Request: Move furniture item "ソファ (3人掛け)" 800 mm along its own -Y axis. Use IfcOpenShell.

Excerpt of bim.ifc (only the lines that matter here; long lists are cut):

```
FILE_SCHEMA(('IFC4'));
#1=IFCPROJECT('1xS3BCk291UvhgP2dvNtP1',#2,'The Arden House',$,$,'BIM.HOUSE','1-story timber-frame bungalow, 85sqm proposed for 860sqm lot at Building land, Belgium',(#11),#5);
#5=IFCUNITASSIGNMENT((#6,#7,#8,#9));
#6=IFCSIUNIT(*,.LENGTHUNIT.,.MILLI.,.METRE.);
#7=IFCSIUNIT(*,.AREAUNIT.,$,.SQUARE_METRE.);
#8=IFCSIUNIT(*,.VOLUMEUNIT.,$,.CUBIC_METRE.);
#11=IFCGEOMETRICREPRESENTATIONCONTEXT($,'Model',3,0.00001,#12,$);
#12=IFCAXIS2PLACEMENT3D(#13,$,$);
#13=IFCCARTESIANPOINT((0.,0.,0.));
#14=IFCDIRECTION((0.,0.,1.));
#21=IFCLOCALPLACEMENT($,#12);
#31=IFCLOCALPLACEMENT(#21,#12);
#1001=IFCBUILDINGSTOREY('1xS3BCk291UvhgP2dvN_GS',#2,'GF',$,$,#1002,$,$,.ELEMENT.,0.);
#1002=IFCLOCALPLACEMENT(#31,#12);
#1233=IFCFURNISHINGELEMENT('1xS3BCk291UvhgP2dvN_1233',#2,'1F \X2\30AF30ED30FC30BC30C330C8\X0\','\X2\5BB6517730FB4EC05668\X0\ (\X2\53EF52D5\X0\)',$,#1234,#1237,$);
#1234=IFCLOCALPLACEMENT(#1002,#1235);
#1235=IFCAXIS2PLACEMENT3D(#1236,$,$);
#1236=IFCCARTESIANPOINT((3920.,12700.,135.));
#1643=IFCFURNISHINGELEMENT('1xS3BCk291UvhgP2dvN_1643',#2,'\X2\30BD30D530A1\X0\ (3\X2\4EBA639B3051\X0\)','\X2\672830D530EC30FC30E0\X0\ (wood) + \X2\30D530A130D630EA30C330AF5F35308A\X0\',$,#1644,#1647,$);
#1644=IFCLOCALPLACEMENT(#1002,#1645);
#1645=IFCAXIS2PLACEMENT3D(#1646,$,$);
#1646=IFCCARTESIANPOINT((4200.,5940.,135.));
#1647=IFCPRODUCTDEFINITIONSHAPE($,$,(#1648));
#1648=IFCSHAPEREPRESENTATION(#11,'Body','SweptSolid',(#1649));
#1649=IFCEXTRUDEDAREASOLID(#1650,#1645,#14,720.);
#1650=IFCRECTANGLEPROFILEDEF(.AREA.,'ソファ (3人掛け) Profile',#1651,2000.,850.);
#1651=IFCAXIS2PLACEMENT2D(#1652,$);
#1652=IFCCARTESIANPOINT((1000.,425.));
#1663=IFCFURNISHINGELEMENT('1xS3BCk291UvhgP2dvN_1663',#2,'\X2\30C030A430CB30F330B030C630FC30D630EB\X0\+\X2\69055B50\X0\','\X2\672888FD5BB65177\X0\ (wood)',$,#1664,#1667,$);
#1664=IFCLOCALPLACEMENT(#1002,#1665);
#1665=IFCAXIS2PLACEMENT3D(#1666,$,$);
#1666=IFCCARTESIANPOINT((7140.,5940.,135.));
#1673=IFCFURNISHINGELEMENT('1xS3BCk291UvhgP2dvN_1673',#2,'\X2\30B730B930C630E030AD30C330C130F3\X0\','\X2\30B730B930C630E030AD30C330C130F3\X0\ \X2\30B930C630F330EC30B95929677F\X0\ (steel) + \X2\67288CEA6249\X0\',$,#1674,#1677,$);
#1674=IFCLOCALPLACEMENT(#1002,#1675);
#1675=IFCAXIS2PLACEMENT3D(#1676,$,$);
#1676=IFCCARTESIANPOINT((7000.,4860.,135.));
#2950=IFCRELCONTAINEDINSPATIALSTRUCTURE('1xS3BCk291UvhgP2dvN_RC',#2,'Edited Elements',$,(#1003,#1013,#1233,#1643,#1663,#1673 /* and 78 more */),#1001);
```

```python
import ifcopenshell
import ifcopenshell.api.geometry
import ifcopenshell.util.placement

model = ifcopenshell.open("bim.ifc")

item = model.by_id(1643)
matrix = ifcopenshell.util.placement.get_local_placement(item.ObjectPlacement)
matrix[:3, 3] -= matrix[:3, 1] * 800.0
ifcopenshell.api.geometry.edit_object_placement(model, product=item, matrix=matrix, is_si=False)

print(ifcopenshell.util.placement.get_local_placement(item.ObjectPlacement).round(3) + 0.0)

model.write("bim_v2.ifc")
```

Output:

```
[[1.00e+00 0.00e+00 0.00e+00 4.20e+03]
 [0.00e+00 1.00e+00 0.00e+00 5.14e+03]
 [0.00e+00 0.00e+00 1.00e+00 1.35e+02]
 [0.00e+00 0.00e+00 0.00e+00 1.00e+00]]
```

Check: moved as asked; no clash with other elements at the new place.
